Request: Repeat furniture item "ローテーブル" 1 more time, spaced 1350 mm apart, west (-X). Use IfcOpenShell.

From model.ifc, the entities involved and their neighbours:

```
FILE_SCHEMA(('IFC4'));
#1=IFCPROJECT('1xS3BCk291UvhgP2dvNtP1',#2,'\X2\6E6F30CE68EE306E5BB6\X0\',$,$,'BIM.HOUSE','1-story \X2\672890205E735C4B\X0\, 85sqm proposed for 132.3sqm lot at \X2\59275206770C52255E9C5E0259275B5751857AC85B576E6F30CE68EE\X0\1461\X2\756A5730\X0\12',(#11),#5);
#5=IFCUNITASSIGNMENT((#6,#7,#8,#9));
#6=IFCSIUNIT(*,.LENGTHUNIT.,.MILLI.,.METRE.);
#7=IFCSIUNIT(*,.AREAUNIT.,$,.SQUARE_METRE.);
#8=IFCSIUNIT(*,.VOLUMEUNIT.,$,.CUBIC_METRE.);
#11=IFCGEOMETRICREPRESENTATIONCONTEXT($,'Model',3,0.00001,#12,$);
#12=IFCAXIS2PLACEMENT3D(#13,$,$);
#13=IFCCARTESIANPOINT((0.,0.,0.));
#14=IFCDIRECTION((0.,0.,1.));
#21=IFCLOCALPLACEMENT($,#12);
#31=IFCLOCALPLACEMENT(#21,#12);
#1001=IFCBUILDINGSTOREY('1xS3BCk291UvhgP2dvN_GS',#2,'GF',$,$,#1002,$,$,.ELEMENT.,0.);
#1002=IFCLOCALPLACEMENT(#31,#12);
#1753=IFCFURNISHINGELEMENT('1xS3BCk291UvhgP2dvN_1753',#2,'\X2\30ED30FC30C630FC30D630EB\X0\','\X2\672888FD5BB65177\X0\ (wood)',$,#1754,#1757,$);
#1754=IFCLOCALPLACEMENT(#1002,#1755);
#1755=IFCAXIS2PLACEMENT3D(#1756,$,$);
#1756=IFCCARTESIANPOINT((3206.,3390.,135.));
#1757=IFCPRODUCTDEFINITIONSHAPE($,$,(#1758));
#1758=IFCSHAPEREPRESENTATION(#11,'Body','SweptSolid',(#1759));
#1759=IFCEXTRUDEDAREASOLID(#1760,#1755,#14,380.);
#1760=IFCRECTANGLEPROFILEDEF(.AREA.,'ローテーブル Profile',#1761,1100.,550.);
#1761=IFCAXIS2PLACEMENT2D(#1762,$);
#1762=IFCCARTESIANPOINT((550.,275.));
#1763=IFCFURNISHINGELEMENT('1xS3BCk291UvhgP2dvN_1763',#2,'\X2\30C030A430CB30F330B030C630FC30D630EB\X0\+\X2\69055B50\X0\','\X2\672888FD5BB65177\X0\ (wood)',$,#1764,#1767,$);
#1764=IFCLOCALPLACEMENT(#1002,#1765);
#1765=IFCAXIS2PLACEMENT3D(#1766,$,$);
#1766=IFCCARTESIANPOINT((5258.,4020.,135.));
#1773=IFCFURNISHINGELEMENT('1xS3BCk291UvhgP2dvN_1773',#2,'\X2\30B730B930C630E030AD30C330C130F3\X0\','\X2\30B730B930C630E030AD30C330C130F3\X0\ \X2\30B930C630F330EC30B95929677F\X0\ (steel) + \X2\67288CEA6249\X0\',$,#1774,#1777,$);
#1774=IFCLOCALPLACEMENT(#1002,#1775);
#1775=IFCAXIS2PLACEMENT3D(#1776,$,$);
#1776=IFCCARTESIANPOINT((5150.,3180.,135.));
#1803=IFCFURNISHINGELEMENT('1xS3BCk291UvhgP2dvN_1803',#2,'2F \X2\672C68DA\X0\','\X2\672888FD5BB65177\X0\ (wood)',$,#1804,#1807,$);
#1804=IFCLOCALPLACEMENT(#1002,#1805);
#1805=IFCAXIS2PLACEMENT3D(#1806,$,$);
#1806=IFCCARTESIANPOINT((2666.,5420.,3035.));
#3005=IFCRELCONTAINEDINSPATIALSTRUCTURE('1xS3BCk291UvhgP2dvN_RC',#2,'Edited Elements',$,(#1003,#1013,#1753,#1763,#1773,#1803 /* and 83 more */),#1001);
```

```python
import numpy as np
import ifcopenshell
import ifcopenshell.api.geometry
import ifcopenshell.api.root
import ifcopenshell.util.element
import ifcopenshell.util.placement
import ifcopenshell.util.unit

model = ifcopenshell.open("model.ifc")
unit_scale = ifcopenshell.util.unit.calculate_unit_scale(model)


def reuse_history(source, copy):
    """copy_class also copies each property set's owner history, people and application; keep the originals."""
    for rel in copy.IsDefinedBy:
        if rel.is_a("IfcRelDefinesByProperties") and (history := rel.RelatingPropertyDefinition.OwnerHistory):
            rel.RelatingPropertyDefinition.OwnerHistory = source.OwnerHistory
            ifcopenshell.util.element.remove_deep2(model, history)


source = model.by_guid("1xS3BCk291UvhgP2dvN_1753")
base = ifcopenshell.util.placement.get_local_placement(source.ObjectPlacement)
step = np.array([-1.0, 0.0, 0.0]) * 1.35 / unit_scale

for i in range(1, 2):
    copy = ifcopenshell.api.root.copy_class(model, product=source)
    copy.Representation = ifcopenshell.util.element.copy_deep(
        model, source.Representation, exclude=["IfcGeometricRepresentationContext", "IfcRepresentationMap"]
    )
    reuse_history(source, copy)
    matrix = base.copy()
    matrix[:3, 3] += i * step
    print("added at", matrix[:3, 3].round(3) + 0.0)
    ifcopenshell.api.geometry.edit_object_placement(model, product=copy, matrix=matrix, is_si=False)

model.write("model_rev.ifc")
```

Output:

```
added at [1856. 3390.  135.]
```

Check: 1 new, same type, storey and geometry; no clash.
